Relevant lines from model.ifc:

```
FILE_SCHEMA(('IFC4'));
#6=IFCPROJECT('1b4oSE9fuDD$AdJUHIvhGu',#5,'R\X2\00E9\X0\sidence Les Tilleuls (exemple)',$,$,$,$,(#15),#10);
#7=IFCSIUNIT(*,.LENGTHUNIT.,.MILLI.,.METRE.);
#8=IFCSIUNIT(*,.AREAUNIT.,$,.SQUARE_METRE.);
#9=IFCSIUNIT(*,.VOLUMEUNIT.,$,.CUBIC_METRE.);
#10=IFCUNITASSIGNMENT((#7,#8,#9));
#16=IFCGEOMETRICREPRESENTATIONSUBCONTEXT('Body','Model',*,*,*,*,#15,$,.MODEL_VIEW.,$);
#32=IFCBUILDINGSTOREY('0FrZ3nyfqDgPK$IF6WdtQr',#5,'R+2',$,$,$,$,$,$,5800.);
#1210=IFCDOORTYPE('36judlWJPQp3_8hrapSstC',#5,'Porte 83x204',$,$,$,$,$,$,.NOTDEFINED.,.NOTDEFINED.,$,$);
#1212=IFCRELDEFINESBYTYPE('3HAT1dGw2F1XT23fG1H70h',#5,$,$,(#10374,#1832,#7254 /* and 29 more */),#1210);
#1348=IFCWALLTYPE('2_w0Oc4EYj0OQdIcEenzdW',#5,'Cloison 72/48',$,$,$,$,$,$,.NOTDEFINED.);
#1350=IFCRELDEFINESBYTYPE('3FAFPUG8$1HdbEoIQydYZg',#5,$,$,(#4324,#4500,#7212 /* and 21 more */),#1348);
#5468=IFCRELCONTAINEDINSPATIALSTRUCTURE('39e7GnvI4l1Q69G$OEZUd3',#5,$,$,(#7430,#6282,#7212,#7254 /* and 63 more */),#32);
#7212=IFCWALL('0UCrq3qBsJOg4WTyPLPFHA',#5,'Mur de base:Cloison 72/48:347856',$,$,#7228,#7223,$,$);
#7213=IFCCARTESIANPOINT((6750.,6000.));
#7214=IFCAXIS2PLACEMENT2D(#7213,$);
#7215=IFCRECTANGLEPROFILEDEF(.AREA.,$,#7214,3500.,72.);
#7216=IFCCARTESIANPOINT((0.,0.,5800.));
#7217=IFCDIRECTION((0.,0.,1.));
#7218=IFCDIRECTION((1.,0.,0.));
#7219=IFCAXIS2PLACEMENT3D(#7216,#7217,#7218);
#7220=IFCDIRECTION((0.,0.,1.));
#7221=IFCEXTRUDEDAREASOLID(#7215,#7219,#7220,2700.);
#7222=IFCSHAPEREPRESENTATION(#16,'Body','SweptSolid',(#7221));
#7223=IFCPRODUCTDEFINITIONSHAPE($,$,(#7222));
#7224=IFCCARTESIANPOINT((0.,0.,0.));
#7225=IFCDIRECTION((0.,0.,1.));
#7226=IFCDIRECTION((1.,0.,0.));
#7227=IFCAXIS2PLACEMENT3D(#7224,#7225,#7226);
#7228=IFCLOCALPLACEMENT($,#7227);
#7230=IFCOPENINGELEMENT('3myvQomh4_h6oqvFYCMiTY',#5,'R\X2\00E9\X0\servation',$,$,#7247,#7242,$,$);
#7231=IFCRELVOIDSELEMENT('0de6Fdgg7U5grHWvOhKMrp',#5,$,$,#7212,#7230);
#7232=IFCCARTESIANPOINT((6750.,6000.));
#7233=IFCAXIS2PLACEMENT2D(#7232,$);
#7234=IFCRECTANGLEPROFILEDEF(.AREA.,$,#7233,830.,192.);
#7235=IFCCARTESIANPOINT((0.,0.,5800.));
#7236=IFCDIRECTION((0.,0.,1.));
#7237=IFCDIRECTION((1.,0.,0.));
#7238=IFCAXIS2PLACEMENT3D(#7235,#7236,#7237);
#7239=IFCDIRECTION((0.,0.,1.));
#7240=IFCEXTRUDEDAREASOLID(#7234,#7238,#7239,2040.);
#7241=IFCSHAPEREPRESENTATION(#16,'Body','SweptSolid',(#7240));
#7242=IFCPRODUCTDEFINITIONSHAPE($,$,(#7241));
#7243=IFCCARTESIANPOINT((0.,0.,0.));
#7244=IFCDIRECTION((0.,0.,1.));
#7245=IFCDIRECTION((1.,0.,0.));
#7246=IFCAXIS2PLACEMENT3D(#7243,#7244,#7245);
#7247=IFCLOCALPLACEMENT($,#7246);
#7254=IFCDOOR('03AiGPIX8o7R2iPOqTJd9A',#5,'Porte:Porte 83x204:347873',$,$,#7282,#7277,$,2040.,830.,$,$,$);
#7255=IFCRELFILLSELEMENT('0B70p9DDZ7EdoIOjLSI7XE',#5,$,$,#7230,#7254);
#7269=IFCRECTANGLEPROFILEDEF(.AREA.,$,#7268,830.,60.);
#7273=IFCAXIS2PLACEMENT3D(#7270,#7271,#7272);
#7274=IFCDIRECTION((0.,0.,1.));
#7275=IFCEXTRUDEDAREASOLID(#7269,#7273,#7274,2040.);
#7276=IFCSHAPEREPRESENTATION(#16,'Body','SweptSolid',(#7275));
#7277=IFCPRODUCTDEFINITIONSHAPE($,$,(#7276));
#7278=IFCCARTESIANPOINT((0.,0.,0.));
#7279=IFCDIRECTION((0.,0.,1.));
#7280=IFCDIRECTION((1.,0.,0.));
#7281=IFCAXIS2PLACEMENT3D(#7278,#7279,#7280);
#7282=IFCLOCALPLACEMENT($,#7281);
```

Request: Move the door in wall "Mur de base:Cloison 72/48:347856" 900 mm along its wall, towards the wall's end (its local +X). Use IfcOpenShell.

```python
import ifcopenshell
import ifcopenshell.api.geometry
import ifcopenshell.util.placement

model = ifcopenshell.open("model.ifc")

door = model.by_id(7254)
opening = door.FillsVoids[0].RelatingOpeningElement
wall = opening.VoidsElements[0].RelatingBuildingElement

wall_matrix = ifcopenshell.util.placement.get_local_placement(wall.ObjectPlacement)
shift = wall_matrix[:3, 0] * 900.0
before = ifcopenshell.util.placement.get_local_placement(door.ObjectPlacement)[:3, 3].copy()

# The door is not placed relative to its opening, so move both.
for product in (opening, door):
    matrix = ifcopenshell.util.placement.get_local_placement(product.ObjectPlacement)
    matrix[:3, 3] += shift
    ifcopenshell.api.geometry.edit_object_placement(model, product=product, matrix=matrix, is_si=False)

after = ifcopenshell.util.placement.get_local_placement(door.ObjectPlacement)[:3, 3]
print("door moved by", (after - before).round(3) + 0.0)

model.write("model_updated.ifc")
```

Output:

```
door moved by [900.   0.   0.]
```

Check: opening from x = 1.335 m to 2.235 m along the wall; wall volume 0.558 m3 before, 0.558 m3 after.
